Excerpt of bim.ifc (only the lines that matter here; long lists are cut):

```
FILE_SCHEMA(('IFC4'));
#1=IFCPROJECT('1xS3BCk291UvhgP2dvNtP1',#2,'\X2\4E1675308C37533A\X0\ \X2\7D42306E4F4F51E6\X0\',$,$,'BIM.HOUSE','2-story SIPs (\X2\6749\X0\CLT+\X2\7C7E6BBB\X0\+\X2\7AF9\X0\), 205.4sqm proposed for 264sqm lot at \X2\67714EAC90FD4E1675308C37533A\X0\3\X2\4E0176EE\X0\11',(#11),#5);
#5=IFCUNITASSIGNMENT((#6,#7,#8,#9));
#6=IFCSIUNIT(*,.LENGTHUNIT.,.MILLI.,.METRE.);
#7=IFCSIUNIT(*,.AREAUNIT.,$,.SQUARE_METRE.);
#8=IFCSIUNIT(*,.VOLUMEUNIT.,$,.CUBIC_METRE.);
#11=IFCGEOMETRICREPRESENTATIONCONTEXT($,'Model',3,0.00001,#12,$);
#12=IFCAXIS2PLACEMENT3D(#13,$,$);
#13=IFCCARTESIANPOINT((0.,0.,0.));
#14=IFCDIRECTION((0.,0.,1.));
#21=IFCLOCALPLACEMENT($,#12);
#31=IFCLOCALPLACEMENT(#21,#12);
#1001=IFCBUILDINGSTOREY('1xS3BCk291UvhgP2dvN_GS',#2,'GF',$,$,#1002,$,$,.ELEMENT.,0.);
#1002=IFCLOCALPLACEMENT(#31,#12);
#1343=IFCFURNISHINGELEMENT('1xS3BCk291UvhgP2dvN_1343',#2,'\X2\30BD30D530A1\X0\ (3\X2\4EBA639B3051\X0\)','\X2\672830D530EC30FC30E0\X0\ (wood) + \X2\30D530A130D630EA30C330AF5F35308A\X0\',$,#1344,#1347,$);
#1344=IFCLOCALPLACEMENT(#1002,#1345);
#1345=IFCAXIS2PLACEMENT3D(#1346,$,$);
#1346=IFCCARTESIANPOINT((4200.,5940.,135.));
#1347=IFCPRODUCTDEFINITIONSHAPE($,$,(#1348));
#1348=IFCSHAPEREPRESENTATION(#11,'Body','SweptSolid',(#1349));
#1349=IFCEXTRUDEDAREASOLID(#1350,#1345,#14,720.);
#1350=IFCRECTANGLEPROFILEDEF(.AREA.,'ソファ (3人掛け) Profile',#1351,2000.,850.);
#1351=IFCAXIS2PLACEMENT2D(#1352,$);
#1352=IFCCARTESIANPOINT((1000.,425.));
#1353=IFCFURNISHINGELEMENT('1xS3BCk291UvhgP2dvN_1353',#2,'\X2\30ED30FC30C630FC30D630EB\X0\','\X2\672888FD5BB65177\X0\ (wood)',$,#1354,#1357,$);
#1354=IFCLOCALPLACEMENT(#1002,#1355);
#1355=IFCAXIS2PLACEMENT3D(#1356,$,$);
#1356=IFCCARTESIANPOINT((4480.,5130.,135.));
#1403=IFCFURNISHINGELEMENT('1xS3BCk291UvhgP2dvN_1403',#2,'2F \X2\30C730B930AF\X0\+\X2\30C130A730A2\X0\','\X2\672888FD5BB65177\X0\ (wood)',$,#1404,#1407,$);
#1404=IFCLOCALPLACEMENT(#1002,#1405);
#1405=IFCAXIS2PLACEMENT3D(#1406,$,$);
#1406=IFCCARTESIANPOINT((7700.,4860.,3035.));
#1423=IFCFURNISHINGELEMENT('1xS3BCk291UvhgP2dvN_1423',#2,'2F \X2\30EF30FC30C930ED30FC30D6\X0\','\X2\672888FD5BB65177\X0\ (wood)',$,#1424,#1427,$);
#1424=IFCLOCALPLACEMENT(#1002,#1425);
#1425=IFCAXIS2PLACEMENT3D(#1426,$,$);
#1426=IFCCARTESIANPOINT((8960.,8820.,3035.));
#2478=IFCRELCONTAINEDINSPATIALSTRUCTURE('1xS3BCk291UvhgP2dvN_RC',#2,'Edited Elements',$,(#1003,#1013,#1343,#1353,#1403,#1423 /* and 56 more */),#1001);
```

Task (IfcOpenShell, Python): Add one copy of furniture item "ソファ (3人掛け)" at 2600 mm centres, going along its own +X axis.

```python
import ifcopenshell
import ifcopenshell.api.geometry
import ifcopenshell.api.root
import ifcopenshell.util.element
import ifcopenshell.util.placement
import ifcopenshell.util.unit

model = ifcopenshell.open("bim.ifc")
unit_scale = ifcopenshell.util.unit.calculate_unit_scale(model)


def reuse_history(source, copy):
    """copy_class also copies each property set's owner history, people and application; keep the originals."""
    for rel in copy.IsDefinedBy:
        if rel.is_a("IfcRelDefinesByProperties") and (history := rel.RelatingPropertyDefinition.OwnerHistory):
            rel.RelatingPropertyDefinition.OwnerHistory = source.OwnerHistory
            ifcopenshell.util.element.remove_deep2(model, history)


source = model.by_guid("1xS3BCk291UvhgP2dvN_1343")
base = ifcopenshell.util.placement.get_local_placement(source.ObjectPlacement)
step = base[:3, 0] * 2.6 / unit_scale

for i in range(1, 2):
    copy = ifcopenshell.api.root.copy_class(model, product=source)
    copy.Representation = ifcopenshell.util.element.copy_deep(
        model, source.Representation, exclude=["IfcGeometricRepresentationContext", "IfcRepresentationMap"]
    )
    reuse_history(source, copy)
    matrix = base.copy()
    matrix[:3, 3] += i * step
    print("added at", matrix[:3, 3].round(3) + 0.0)
    ifcopenshell.api.geometry.edit_object_placement(model, product=copy, matrix=matrix, is_si=False)

model.write("bim_updated.ifc")
```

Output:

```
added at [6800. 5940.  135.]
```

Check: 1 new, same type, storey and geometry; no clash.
